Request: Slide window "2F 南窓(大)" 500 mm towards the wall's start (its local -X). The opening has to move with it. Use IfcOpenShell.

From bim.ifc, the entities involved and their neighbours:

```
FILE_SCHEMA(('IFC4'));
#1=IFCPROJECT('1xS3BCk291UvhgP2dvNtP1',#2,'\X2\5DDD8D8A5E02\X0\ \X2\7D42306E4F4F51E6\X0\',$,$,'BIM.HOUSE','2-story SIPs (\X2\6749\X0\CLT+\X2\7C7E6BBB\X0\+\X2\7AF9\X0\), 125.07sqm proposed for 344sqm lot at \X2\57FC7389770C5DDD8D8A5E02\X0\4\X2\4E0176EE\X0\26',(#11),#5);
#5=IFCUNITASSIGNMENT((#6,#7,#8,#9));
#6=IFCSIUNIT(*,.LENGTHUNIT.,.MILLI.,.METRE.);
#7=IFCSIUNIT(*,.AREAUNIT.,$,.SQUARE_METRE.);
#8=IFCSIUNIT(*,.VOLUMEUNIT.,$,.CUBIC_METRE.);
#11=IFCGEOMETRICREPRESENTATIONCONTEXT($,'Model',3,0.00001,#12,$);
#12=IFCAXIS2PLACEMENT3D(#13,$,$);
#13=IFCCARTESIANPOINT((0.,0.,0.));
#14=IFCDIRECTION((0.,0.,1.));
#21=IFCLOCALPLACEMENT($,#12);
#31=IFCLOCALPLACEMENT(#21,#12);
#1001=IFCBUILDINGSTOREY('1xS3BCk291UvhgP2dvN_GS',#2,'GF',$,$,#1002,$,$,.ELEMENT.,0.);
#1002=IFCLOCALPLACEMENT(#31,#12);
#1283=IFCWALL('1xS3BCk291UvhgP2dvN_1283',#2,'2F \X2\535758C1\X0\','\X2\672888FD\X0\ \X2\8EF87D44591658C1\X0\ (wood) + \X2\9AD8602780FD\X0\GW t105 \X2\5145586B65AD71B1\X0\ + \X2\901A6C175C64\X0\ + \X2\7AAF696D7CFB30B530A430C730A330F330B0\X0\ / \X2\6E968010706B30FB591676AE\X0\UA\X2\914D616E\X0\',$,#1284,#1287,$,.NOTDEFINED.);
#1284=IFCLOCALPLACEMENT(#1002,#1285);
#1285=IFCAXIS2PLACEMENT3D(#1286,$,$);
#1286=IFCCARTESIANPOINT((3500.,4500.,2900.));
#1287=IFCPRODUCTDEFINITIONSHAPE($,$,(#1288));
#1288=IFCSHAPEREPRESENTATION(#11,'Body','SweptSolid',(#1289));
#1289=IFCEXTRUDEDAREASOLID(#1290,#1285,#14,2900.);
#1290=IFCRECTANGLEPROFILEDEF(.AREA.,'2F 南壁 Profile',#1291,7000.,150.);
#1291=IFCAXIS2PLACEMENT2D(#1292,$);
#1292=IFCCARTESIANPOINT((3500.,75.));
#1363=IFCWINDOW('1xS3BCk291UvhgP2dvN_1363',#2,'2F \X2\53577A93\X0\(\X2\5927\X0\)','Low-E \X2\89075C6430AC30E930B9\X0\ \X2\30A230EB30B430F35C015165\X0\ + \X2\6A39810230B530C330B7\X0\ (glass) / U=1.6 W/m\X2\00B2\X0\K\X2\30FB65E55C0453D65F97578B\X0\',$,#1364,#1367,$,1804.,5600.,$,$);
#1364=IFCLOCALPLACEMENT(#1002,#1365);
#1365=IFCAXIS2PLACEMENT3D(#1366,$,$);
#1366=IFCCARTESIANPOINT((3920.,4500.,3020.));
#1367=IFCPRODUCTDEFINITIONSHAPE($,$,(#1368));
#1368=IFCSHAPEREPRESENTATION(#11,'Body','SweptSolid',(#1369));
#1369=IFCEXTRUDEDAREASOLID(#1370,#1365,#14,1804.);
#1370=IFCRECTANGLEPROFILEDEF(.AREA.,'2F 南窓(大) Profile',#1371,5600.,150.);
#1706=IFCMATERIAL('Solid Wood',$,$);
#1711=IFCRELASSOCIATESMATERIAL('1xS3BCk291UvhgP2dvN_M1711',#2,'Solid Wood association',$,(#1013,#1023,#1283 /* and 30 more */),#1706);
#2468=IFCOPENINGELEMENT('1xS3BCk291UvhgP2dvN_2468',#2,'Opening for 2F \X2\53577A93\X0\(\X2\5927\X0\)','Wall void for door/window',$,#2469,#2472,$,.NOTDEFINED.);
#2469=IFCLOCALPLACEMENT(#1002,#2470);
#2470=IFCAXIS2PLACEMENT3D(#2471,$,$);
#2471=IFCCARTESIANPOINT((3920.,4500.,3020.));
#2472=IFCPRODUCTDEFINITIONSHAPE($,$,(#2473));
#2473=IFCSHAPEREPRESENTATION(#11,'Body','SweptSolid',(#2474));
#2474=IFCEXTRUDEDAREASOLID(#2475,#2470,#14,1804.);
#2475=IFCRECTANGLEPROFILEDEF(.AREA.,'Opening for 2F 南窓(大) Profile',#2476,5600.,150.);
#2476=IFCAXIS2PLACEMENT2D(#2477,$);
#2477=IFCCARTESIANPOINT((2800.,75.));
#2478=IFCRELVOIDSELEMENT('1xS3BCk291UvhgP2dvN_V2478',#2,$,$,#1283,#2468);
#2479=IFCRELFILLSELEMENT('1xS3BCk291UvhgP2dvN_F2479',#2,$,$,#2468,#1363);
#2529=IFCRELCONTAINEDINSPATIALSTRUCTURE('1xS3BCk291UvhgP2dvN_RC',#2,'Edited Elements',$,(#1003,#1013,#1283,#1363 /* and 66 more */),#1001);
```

```python
import ifcopenshell
import ifcopenshell.api.geometry
import ifcopenshell.util.placement

model = ifcopenshell.open("bim.ifc")

window = model.by_guid("1xS3BCk291UvhgP2dvN_1363")
opening = window.FillsVoids[0].RelatingOpeningElement
wall = opening.VoidsElements[0].RelatingBuildingElement

wall_matrix = ifcopenshell.util.placement.get_local_placement(wall.ObjectPlacement)
shift = wall_matrix[:3, 0] * -500.0
before = ifcopenshell.util.placement.get_local_placement(window.ObjectPlacement)[:3, 3].copy()

# The window is not placed relative to its opening, so move both.
for product in (opening, window):
    matrix = ifcopenshell.util.placement.get_local_placement(product.ObjectPlacement)
    matrix[:3, 3] += shift
    ifcopenshell.api.geometry.edit_object_placement(model, product=product, matrix=matrix, is_si=False)

after = ifcopenshell.util.placement.get_local_placement(window.ObjectPlacement)[:3, 3]
print("window moved by", (after - before).round(3) + 0.0)

model.write("bim_rev.ifc")
```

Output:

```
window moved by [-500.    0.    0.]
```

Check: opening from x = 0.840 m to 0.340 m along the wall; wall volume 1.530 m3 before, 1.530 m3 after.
